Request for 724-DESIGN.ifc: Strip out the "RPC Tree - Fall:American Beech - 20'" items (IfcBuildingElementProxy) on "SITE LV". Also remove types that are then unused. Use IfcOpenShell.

First a look at what the model holds.

```python
import ifcopenshell
import ifcopenshell.util.element

model = ifcopenshell.open("724-DESIGN.ifc")
print(model.schema)
storey = next(s for s in model.by_type("IfcBuildingStorey") if s.Name == "SITE LV")
proxies = [e for e in ifcopenshell.util.element.get_decomposition(storey) if e.is_a("IfcBuildingElementProxy")]
seen = {}
for e in proxies:
    element_type = ifcopenshell.util.element.get_type(e)
    name = element_type.Name if element_type not in (None, e) else None
    seen[name] = seen.get(name, 0) + 1
for name, count in sorted(seen.items(), key=str):
    print(count, "x", name)
```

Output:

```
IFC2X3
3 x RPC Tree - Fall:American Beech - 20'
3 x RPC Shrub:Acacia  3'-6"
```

```python
import ifcopenshell
import ifcopenshell.api.root
import ifcopenshell.util.element

model = ifcopenshell.open("724-DESIGN.ifc")

storey = next(s for s in model.by_type("IfcBuildingStorey") if s.Name == "SITE LV")
proxies = [e for e in ifcopenshell.util.element.get_decomposition(storey) if e.is_a("IfcBuildingElementProxy")]
targets = [e for e in proxies if (t := ifcopenshell.util.element.get_type(e)) not in (None, e) and t.Name == "RPC Tree - Fall:American Beech - 20'"]
types = {ifcopenshell.util.element.get_type(e) for e in targets} - {None, *targets}

for e in targets:
    ifcopenshell.api.root.remove_product(model, product=e)
print(len(targets), "removed")

unused = [t for t in types if not ifcopenshell.util.element.get_types(t)]
for t in unused:
    ifcopenshell.api.root.remove_product(model, product=t)
print(len(unused), "unused types removed")

model.write("724-DESIGN_rev.ifc")
```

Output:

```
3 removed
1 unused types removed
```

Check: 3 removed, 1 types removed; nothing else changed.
